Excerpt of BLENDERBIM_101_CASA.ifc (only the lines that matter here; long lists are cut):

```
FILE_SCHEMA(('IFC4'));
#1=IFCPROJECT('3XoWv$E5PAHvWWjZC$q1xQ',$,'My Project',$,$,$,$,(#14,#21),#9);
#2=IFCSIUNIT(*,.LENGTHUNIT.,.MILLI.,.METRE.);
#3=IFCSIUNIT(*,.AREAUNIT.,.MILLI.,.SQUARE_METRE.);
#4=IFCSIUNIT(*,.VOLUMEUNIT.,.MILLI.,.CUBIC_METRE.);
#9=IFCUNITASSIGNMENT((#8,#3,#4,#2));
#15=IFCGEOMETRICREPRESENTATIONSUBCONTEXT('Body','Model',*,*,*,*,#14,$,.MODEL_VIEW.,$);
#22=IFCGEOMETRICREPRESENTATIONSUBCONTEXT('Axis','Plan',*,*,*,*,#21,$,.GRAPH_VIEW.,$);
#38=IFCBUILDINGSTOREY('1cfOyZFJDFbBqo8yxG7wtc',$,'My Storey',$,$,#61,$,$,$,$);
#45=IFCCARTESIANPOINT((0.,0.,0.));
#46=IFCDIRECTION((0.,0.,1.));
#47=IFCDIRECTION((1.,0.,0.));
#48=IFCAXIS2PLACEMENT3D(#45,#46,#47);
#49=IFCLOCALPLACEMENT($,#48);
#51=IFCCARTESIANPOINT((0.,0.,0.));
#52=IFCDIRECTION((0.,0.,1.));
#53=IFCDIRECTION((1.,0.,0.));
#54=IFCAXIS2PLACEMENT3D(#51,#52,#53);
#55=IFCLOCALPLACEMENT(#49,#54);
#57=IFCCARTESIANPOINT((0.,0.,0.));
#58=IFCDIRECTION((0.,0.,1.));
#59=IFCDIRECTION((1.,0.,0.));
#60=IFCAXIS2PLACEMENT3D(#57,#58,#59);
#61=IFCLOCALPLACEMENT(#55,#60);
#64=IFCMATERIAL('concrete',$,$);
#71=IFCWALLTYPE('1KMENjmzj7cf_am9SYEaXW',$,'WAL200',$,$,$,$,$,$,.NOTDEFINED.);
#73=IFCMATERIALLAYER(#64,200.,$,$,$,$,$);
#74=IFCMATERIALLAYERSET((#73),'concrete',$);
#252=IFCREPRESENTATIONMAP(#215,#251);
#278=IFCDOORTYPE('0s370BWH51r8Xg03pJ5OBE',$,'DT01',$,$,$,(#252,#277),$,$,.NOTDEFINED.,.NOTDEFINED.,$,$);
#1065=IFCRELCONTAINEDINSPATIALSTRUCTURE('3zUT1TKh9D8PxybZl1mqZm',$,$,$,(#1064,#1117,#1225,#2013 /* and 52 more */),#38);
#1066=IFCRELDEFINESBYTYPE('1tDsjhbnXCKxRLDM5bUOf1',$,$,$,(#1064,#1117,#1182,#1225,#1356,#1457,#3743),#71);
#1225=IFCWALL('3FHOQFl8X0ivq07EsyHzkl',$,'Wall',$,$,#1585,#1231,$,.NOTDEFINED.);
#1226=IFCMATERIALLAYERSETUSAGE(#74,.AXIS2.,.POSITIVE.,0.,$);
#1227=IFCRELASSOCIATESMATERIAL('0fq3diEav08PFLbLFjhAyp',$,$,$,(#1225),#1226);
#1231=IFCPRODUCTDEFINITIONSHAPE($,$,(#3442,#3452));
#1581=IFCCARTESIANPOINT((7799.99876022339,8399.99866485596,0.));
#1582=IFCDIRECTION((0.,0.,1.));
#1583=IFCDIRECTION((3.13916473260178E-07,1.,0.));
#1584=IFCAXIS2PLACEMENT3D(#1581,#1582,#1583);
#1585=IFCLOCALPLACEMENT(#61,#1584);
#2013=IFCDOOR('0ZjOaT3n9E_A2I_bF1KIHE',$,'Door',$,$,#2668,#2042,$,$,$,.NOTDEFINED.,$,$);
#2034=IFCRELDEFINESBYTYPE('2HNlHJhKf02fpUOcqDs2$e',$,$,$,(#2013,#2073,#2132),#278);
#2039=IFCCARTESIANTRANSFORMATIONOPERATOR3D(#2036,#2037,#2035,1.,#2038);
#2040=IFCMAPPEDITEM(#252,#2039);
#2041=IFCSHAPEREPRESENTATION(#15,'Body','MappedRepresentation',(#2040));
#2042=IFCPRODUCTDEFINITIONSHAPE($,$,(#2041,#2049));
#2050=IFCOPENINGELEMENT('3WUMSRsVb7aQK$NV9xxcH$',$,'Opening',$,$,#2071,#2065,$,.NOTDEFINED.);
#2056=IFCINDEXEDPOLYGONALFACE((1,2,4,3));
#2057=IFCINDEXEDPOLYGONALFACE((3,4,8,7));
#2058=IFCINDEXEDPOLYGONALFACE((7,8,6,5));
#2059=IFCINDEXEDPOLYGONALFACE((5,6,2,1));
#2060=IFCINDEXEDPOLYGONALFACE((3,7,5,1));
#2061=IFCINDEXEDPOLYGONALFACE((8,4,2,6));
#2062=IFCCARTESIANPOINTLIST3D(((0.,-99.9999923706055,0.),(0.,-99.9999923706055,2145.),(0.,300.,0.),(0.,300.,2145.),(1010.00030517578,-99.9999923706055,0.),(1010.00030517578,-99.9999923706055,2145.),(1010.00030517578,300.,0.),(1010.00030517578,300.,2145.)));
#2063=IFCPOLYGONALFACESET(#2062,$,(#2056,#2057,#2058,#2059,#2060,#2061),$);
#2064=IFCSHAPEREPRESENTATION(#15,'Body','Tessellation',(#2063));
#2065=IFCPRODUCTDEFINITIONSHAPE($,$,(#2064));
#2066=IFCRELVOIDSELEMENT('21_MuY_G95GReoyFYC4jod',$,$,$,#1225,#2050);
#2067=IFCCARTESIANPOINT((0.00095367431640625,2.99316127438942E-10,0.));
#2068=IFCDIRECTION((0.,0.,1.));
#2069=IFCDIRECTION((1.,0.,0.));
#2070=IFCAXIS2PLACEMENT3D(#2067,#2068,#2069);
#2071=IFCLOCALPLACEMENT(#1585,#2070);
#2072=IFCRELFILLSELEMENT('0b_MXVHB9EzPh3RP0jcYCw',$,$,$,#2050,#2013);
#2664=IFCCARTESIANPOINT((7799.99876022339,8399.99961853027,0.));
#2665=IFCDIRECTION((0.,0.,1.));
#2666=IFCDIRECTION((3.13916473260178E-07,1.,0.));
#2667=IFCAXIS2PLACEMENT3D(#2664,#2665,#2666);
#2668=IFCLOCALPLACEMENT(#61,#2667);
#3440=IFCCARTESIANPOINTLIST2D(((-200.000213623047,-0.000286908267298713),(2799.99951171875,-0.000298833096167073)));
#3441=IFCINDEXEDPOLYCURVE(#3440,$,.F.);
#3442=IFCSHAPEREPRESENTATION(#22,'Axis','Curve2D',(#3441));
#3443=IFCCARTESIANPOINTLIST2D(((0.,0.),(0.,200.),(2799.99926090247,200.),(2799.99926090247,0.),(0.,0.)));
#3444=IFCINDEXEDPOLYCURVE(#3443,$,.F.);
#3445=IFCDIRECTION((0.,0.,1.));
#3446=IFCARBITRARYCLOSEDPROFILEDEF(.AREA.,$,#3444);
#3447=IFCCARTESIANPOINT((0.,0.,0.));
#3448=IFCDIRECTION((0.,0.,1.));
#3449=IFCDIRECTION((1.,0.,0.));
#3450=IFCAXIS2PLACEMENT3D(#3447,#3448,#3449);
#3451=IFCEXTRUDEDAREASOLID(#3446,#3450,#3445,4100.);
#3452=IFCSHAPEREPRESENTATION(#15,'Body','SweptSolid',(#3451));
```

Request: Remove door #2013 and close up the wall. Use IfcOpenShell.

```python
import ifcopenshell
import ifcopenshell.api.feature
import ifcopenshell.api.root
import ifcopenshell.geom
import ifcopenshell.util.shape

model = ifcopenshell.open("BLENDERBIM_101_CASA.ifc")
settings = ifcopenshell.geom.settings()


def volume(element):
    """Net volume in cubic metres, openings subtracted."""
    shape = ifcopenshell.geom.create_shape(settings, element)
    return ifcopenshell.util.shape.get_volume(shape.geometry)


door = model.by_id(2013)
opening = door.FillsVoids[0].RelatingOpeningElement
wall = opening.VoidsElements[0].RelatingBuildingElement
before = volume(wall)

ifcopenshell.api.root.remove_product(model, product=door)
ifcopenshell.api.feature.remove_feature(model, feature=opening)

after = volume(wall)

print(f"wall volume {before:.3f} -> {after:.3f} m3")

model.write("BLENDERBIM_101_CASA-out.ifc")
```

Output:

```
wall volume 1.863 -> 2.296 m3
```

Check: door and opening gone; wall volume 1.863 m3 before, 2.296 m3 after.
